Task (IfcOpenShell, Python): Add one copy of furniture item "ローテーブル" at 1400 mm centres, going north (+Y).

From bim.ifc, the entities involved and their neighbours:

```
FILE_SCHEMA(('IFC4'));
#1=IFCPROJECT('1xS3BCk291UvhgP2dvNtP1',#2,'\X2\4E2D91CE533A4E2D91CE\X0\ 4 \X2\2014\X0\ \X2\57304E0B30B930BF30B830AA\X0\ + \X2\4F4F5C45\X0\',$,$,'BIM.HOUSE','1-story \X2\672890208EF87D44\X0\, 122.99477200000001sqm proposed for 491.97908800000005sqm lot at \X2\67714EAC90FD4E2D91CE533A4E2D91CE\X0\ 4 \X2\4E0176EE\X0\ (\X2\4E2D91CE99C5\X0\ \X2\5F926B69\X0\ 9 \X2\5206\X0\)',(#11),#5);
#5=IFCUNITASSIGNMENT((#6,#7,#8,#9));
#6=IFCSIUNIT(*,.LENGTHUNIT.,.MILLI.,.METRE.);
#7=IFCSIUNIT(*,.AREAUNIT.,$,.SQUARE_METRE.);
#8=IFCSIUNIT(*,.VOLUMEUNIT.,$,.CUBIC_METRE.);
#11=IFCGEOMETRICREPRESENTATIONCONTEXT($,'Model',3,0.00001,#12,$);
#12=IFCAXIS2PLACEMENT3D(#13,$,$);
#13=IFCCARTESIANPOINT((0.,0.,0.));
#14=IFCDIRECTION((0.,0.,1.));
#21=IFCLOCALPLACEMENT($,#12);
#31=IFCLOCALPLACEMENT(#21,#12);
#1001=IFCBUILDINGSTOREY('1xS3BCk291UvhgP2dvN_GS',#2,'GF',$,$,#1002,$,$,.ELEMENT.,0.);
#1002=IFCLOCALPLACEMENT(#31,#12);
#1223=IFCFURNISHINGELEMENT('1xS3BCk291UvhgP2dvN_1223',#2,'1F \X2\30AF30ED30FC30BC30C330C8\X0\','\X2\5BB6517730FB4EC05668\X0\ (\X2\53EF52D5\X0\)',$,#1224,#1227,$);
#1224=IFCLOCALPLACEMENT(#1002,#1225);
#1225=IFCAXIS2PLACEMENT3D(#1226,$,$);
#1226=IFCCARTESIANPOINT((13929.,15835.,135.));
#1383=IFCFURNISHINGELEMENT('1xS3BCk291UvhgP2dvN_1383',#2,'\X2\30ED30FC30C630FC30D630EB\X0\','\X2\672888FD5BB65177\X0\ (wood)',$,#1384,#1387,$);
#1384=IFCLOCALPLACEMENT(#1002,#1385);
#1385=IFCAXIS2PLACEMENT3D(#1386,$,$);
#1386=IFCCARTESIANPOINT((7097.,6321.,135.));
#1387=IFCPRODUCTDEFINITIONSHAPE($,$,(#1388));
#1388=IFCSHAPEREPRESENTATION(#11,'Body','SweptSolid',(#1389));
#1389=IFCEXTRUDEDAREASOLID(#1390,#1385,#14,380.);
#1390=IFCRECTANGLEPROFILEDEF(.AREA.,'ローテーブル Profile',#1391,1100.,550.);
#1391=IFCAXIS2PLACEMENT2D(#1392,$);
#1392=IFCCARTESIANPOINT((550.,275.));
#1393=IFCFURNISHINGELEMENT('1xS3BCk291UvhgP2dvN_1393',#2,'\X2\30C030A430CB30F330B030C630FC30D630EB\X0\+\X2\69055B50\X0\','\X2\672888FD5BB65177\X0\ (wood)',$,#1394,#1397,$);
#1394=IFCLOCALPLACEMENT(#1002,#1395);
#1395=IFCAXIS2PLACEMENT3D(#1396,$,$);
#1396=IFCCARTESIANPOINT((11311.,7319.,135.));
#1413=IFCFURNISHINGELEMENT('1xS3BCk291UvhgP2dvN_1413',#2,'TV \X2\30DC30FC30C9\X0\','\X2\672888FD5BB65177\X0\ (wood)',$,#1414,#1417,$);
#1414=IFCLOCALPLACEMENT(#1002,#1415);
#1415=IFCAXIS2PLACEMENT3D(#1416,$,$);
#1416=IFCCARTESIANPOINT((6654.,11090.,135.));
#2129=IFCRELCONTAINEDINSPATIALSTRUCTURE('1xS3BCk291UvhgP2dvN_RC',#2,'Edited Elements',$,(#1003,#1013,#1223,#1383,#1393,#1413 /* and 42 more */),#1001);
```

```python
import numpy as np
import ifcopenshell
import ifcopenshell.api.geometry
import ifcopenshell.api.root
import ifcopenshell.util.element
import ifcopenshell.util.placement

model = ifcopenshell.open("bim.ifc")


def reuse_history(source, copy):
    """copy_class also copies each property set's owner history, people and application; keep the originals."""
    for rel in copy.IsDefinedBy:
        if rel.is_a("IfcRelDefinesByProperties") and (history := rel.RelatingPropertyDefinition.OwnerHistory):
            rel.RelatingPropertyDefinition.OwnerHistory = source.OwnerHistory
            ifcopenshell.util.element.remove_deep2(model, history)


source = model.by_guid("1xS3BCk291UvhgP2dvN_1383")
base = ifcopenshell.util.placement.get_local_placement(source.ObjectPlacement)
step = np.array([0.0, 1.0, 0.0]) * 1400.0

for i in range(1, 2):
    copy = ifcopenshell.api.root.copy_class(model, product=source)
    copy.Representation = ifcopenshell.util.element.copy_deep(
        model, source.Representation, exclude=["IfcGeometricRepresentationContext", "IfcRepresentationMap"]
    )
    reuse_history(source, copy)
    matrix = base.copy()
    matrix[:3, 3] += i * step
    print("added at", matrix[:3, 3].round(3) + 0.0)
    ifcopenshell.api.geometry.edit_object_placement(model, product=copy, matrix=matrix, is_si=False)

model.write("bim-out.ifc")
```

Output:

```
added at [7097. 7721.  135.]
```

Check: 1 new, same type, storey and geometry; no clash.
